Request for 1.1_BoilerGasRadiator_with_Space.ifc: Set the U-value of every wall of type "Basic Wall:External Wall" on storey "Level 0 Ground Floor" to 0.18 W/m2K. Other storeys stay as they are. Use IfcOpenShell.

First a look at what the model holds.

```python
import ifcopenshell
import ifcopenshell.util.element

model = ifcopenshell.open("1.1_BoilerGasRadiator_with_Space.ifc")
print(model.schema)
storey = next(s for s in model.by_type("IfcBuildingStorey") if s.Name == "Level 0 Ground Floor")
walls = [e for e in ifcopenshell.util.element.get_decomposition(storey) if e.is_a("IfcWall")]
seen = {}
for e in walls:
    element_type = ifcopenshell.util.element.get_type(e)
    key = (element_type.Name if element_type != e and element_type else None, ifcopenshell.util.element.get_pset(e, "Pset_WallCommon", "ThermalTransmittance"))
    seen[key] = seen.get(key, 0) + 1
for (name, value), count in sorted(seen.items(), key=str):
    print(count, "x", name, "|", value)
```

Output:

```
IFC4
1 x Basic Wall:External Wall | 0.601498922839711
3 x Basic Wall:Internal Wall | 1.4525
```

```python
import ifcopenshell
import ifcopenshell.api.pset
import ifcopenshell.util.element

model = ifcopenshell.open("1.1_BoilerGasRadiator_with_Space.ifc")

storey = next(s for s in model.by_type("IfcBuildingStorey") if s.Name == "Level 0 Ground Floor")
walls = [e for e in ifcopenshell.util.element.get_decomposition(storey) if e.is_a("IfcWall")]

count = 0
for e in walls:
    element_type = ifcopenshell.util.element.get_type(e)
    if element_type in (None, e) or element_type.Name != "Basic Wall:External Wall":
        continue
    # add_pset returns the element's existing set when there is one.
    pset = ifcopenshell.api.pset.add_pset(model, product=e, name="Pset_WallCommon")
    ifcopenshell.api.pset.edit_pset(model, pset=pset, properties={"ThermalTransmittance": 0.18})
    count += 1

print(count, "walls updated")

model.write("1.1_BoilerGasRadiator_with_Space_edited.ifc")
```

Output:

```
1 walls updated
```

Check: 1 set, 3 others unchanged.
